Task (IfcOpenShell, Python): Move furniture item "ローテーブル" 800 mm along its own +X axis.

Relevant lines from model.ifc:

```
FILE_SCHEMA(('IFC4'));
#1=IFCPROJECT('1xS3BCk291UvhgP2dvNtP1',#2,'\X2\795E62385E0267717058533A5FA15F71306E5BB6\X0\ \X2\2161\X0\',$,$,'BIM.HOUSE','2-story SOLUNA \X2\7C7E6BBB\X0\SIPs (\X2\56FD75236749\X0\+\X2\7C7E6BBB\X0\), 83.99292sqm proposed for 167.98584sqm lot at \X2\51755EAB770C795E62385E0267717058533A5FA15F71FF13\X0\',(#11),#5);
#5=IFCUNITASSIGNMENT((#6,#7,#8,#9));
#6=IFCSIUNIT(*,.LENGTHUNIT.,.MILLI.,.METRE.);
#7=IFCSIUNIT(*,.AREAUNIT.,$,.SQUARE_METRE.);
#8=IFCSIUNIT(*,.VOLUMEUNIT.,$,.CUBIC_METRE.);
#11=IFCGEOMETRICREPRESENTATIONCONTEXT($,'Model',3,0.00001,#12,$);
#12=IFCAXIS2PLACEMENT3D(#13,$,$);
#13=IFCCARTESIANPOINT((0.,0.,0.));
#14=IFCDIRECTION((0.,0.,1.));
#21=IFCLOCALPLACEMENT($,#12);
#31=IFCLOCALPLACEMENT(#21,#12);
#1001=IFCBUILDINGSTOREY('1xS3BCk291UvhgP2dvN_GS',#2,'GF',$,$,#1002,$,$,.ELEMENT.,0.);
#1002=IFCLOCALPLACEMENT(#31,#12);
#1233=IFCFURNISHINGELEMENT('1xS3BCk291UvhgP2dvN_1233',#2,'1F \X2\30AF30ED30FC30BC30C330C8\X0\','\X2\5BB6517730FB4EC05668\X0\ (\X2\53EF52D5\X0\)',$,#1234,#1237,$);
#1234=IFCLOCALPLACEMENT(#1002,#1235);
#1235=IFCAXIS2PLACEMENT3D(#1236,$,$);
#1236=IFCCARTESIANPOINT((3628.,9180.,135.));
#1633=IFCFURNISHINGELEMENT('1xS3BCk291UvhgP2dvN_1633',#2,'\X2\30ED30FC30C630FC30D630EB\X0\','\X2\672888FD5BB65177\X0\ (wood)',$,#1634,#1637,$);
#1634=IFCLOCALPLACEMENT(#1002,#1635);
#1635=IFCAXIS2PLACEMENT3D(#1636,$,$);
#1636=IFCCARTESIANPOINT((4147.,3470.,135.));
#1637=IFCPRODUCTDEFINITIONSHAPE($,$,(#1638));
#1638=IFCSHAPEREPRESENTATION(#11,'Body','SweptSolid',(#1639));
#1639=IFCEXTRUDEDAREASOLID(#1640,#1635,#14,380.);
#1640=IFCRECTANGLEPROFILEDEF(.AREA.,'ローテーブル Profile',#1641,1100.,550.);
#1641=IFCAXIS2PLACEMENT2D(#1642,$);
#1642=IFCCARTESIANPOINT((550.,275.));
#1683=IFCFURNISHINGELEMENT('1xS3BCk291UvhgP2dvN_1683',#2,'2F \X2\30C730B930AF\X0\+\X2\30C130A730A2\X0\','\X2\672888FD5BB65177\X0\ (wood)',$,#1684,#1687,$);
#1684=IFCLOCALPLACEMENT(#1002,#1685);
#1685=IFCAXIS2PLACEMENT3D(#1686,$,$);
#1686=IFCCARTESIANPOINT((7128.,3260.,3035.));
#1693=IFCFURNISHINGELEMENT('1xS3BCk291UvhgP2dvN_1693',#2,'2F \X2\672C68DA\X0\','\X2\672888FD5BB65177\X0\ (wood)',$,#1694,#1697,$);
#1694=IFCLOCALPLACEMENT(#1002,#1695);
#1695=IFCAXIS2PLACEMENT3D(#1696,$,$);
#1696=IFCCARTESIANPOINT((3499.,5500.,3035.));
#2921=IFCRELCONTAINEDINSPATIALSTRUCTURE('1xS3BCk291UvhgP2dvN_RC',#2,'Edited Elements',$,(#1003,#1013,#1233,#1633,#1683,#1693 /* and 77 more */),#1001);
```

```python
import ifcopenshell
import ifcopenshell.api.geometry
import ifcopenshell.util.placement
import ifcopenshell.util.unit

model = ifcopenshell.open("model.ifc")
unit_scale = ifcopenshell.util.unit.calculate_unit_scale(model)

item = model.by_guid("1xS3BCk291UvhgP2dvN_1633")
matrix = ifcopenshell.util.placement.get_local_placement(item.ObjectPlacement)
matrix[:3, 3] += matrix[:3, 0] * 0.8 / unit_scale
ifcopenshell.api.geometry.edit_object_placement(model, product=item, matrix=matrix, is_si=False)

print(ifcopenshell.util.placement.get_local_placement(item.ObjectPlacement).round(3) + 0.0)

model.write("model-out.ifc")
```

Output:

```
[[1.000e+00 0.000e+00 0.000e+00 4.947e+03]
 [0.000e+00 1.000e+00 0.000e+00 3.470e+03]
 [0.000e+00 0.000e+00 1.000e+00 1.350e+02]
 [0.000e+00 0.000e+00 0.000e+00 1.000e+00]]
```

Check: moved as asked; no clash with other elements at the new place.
